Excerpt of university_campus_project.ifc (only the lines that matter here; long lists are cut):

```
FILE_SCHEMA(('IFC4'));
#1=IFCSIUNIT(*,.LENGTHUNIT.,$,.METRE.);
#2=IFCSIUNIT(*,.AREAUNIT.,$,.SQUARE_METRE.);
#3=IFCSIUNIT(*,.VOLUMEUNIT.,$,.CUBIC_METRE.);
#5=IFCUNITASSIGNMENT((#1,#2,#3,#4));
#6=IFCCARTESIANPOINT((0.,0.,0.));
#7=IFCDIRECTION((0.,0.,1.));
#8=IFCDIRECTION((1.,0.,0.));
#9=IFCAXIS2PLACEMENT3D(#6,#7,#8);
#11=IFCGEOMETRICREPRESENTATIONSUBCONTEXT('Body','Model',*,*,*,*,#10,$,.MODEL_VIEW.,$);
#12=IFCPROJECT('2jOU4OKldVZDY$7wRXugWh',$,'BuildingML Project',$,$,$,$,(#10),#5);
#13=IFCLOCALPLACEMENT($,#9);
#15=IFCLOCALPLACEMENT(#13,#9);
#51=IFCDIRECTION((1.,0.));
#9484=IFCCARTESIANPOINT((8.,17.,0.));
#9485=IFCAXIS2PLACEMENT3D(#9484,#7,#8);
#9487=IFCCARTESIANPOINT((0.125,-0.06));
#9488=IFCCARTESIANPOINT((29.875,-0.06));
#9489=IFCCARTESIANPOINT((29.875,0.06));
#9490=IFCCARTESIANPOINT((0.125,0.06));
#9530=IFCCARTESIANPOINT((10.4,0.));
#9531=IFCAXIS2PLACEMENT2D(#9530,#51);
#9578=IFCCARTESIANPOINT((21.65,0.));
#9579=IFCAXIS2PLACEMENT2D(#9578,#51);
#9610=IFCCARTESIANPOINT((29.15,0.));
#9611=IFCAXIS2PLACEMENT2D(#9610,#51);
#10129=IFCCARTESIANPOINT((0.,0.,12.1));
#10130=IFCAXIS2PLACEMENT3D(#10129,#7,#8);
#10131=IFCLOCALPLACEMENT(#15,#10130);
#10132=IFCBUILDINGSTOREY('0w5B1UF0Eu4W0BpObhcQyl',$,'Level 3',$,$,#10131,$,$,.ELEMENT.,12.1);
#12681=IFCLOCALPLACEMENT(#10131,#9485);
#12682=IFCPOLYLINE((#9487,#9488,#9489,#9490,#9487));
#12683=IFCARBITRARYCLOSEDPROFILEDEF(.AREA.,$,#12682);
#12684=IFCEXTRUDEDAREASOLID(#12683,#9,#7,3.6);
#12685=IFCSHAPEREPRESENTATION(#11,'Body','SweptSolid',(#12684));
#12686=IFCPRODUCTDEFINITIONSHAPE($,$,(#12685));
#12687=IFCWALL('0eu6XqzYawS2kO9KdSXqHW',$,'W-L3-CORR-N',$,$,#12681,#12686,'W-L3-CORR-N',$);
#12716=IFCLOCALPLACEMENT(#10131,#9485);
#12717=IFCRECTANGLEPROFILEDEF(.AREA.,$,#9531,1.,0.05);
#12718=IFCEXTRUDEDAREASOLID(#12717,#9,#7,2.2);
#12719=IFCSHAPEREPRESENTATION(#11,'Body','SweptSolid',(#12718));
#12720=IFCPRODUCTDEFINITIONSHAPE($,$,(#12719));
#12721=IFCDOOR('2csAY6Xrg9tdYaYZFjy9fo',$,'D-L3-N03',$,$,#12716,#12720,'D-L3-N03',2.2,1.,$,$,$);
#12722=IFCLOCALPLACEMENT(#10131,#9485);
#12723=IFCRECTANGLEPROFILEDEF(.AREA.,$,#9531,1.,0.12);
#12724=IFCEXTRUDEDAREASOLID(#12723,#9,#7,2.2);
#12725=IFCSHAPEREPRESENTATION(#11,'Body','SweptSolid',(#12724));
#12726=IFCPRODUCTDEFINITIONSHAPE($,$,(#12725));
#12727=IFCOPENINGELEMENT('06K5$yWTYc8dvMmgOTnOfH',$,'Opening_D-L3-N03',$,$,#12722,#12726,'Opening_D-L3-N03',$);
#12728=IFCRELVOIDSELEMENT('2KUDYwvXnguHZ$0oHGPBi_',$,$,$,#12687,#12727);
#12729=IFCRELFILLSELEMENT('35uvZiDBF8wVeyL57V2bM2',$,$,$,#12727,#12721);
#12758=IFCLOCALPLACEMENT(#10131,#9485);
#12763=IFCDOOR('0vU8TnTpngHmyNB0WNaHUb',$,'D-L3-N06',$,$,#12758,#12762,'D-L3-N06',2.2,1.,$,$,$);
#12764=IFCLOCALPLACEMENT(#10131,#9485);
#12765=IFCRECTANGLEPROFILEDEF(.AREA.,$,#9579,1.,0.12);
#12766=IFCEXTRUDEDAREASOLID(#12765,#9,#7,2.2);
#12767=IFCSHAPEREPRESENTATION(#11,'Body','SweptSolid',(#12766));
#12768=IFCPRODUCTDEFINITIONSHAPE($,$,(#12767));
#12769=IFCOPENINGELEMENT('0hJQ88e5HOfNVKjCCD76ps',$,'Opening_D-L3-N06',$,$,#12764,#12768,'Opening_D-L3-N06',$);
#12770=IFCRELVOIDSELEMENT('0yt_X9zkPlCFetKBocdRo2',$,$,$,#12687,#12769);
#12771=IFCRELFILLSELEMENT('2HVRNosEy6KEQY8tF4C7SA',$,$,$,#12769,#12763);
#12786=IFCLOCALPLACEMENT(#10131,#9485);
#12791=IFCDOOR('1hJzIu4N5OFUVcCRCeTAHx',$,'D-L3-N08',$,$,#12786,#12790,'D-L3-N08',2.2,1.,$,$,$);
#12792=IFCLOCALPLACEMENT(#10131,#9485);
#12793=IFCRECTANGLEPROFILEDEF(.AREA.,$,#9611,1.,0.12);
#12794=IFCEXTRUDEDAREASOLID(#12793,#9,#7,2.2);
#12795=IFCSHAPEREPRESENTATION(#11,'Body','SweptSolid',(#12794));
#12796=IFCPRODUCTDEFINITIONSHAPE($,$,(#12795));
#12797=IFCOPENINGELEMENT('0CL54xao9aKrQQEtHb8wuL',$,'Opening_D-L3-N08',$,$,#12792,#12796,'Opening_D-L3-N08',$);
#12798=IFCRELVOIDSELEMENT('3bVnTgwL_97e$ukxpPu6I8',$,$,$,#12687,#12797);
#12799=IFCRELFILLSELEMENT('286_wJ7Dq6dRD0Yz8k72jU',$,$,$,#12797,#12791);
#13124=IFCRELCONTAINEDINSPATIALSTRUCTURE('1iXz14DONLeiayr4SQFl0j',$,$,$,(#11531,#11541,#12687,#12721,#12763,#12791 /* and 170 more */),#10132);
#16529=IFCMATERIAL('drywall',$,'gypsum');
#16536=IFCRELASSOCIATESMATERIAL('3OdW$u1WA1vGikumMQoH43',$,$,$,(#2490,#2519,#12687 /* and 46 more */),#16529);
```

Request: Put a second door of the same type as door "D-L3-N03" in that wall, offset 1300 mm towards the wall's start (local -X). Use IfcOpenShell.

```python
import ifcopenshell
import ifcopenshell.api.feature
import ifcopenshell.api.geometry
import ifcopenshell.api.root
import ifcopenshell.geom
import ifcopenshell.util.element
import ifcopenshell.util.placement
import ifcopenshell.util.shape
import ifcopenshell.util.unit

model = ifcopenshell.open("university_campus_project.ifc")
unit_scale = ifcopenshell.util.unit.calculate_unit_scale(model)
settings = ifcopenshell.geom.settings()


def volume(element):
    """Net volume in cubic metres, openings subtracted."""
    shape = ifcopenshell.geom.create_shape(settings, element)
    return ifcopenshell.util.shape.get_volume(shape.geometry)


door = model.by_guid("2csAY6Xrg9tdYaYZFjy9fo")
opening = door.FillsVoids[0].RelatingOpeningElement
wall = opening.VoidsElements[0].RelatingBuildingElement
before = volume(wall)
shift = ifcopenshell.util.placement.get_local_placement(wall.ObjectPlacement)[:3, 0] * -1.3 / unit_scale

# copy_class copies the void relationship, type, container and properties, but no geometry.
new_opening = ifcopenshell.api.root.copy_class(model, product=opening)
new_opening.Representation = ifcopenshell.util.element.copy_deep(
    model, opening.Representation, exclude=["IfcGeometricRepresentationContext", "IfcRepresentationMap"]
)
new_opening.Tag = None
new_door = ifcopenshell.api.root.copy_class(model, product=door)
new_door.Representation = ifcopenshell.util.element.copy_deep(
    model, door.Representation, exclude=["IfcGeometricRepresentationContext", "IfcRepresentationMap"]
)
new_door.Tag = None
ifcopenshell.api.feature.add_filling(model, opening=new_opening, element=new_door)

for old, new in ((opening, new_opening), (door, new_door)):
    matrix = ifcopenshell.util.placement.get_local_placement(old.ObjectPlacement)
    matrix[:3, 3] += shift
    ifcopenshell.api.geometry.edit_object_placement(model, product=new, matrix=matrix, is_si=False)

after = volume(wall)

print(f"wall volume {before:.3f} -> {after:.3f} m3")

model.write("university_campus_project_updated.ifc")
```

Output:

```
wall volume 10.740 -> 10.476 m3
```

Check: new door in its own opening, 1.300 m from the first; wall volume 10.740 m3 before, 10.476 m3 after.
